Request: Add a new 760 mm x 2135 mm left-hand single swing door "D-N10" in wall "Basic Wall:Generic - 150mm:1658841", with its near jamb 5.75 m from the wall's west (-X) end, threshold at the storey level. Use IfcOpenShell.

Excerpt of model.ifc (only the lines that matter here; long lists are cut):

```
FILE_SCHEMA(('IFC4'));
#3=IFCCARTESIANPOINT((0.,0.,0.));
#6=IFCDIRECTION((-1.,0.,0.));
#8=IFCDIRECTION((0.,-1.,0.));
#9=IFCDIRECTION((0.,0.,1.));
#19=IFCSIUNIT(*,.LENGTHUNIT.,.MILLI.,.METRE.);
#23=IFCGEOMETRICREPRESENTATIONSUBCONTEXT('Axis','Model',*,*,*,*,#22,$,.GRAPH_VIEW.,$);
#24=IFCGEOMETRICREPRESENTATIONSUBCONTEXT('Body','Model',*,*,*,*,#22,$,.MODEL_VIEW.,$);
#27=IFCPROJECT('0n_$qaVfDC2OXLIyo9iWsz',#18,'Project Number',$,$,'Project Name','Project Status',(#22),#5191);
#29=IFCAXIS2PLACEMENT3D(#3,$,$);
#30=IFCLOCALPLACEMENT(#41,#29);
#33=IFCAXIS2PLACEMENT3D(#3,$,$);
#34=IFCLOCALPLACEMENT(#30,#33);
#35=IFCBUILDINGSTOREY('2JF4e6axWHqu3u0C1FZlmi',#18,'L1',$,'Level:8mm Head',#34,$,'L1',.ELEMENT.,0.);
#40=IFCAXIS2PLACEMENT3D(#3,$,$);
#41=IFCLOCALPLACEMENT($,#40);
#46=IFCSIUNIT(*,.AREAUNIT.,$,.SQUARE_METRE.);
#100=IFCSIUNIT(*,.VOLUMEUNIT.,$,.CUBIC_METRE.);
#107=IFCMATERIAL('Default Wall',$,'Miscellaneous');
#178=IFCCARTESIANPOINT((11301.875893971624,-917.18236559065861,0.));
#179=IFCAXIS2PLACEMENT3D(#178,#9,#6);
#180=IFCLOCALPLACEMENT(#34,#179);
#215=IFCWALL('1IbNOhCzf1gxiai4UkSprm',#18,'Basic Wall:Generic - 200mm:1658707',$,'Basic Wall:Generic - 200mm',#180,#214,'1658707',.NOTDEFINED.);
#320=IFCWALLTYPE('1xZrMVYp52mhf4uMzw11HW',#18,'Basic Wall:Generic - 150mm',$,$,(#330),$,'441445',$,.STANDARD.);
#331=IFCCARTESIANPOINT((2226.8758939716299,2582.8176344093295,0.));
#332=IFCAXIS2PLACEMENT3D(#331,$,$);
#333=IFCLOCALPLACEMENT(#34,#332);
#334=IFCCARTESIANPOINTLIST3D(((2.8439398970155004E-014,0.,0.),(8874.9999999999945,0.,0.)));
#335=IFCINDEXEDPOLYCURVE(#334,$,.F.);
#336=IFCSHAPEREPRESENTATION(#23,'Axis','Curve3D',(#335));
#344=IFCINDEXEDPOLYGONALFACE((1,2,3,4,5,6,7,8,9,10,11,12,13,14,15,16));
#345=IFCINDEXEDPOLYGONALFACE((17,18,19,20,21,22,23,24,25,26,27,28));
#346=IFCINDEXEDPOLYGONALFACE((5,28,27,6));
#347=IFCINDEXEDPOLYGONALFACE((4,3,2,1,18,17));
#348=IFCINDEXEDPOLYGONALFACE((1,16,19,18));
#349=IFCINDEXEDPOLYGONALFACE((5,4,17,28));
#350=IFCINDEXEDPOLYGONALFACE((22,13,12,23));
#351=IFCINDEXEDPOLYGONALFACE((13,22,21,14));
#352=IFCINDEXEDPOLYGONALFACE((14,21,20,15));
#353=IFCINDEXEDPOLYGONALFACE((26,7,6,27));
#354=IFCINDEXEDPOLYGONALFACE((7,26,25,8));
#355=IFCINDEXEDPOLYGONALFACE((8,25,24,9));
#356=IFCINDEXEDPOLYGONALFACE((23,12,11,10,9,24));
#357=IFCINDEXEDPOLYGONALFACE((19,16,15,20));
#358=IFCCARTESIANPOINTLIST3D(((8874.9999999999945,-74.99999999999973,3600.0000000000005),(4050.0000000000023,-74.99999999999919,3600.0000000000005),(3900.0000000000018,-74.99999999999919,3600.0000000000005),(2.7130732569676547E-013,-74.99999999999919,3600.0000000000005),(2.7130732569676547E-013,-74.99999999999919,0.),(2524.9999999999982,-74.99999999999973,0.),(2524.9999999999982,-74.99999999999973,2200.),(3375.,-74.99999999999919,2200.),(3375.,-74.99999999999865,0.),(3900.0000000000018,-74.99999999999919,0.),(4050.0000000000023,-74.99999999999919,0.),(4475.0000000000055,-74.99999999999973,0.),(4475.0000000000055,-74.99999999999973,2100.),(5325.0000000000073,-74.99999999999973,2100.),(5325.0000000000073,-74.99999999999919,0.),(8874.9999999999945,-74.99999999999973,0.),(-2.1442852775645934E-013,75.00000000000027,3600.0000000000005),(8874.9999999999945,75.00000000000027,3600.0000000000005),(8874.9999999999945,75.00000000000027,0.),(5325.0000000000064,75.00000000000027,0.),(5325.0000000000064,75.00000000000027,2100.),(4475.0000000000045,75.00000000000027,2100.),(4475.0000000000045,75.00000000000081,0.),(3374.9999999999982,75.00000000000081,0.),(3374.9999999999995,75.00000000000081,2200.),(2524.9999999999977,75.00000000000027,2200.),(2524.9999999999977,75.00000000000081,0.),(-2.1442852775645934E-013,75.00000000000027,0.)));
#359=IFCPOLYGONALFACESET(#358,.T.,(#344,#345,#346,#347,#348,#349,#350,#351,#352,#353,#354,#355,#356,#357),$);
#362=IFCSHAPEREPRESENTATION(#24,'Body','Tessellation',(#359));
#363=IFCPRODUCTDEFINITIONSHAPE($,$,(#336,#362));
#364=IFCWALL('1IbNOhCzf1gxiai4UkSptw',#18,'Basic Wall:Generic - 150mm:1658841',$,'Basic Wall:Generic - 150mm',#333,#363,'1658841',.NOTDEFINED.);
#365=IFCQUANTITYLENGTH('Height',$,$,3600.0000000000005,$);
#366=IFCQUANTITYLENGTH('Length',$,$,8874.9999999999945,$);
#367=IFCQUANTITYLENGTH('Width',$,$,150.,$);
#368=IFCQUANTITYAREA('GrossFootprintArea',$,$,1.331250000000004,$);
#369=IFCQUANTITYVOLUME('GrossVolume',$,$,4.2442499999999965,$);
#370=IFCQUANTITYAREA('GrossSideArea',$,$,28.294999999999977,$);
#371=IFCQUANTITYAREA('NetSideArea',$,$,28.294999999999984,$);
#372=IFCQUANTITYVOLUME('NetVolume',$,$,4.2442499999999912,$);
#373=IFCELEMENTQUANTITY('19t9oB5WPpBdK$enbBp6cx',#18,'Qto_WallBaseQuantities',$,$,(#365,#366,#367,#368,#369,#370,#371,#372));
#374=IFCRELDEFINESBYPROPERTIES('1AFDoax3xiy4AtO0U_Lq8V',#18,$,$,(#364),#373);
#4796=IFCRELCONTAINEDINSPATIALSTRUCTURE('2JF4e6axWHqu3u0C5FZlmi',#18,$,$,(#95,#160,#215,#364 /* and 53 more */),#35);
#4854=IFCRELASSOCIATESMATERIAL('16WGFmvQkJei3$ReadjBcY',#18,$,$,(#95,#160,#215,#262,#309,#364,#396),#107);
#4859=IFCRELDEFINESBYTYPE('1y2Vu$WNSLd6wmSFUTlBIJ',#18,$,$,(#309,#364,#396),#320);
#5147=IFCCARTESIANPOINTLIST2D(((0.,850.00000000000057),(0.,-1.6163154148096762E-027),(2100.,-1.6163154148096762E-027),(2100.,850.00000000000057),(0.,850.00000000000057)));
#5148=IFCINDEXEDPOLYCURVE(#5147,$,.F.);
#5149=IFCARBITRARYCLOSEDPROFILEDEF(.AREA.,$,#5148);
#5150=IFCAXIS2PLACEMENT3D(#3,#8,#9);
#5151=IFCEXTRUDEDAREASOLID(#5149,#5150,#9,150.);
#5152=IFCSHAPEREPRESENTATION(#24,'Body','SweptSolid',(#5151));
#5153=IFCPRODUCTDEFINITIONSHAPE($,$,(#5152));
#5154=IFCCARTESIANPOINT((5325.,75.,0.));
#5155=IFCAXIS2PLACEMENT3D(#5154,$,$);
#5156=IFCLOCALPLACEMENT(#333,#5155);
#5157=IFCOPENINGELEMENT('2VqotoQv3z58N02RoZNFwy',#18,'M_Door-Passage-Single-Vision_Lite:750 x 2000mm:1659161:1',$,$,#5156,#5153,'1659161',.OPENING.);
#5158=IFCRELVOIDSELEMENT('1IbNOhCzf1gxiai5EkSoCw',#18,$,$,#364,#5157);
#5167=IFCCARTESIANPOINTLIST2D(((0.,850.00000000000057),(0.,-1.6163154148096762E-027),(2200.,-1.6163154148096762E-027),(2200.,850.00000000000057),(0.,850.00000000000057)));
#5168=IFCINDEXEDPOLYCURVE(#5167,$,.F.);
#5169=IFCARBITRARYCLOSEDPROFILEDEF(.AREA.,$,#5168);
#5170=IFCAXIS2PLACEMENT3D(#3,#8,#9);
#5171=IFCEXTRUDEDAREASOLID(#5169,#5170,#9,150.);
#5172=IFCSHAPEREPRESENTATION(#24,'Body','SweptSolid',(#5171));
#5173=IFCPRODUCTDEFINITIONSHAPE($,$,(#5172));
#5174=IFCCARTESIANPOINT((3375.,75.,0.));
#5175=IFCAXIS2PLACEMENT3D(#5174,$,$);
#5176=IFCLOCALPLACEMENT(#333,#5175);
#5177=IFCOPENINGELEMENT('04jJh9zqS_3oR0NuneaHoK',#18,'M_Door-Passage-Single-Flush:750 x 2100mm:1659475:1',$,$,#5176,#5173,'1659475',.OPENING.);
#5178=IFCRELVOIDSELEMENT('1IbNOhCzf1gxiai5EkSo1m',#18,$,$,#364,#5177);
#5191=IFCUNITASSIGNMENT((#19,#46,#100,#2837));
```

```python
import numpy as np
import ifcopenshell
import ifcopenshell.api.feature
import ifcopenshell.api.geometry
import ifcopenshell.api.pset
import ifcopenshell.api.root
import ifcopenshell.api.spatial
import ifcopenshell.geom
import ifcopenshell.util.element
import ifcopenshell.util.placement
import ifcopenshell.util.representation
import ifcopenshell.util.shape
import ifcopenshell.util.unit

model = ifcopenshell.open("model.ifc")
unit_scale = ifcopenshell.util.unit.calculate_unit_scale(model)
area_scale = ifcopenshell.util.unit.calculate_unit_scale(model, "AREAUNIT")
volume_scale = ifcopenshell.util.unit.calculate_unit_scale(model, "VOLUMEUNIT")
settings = ifcopenshell.geom.settings()


def volume(element):
    """Net volume in cubic metres, openings subtracted."""
    shape = ifcopenshell.geom.create_shape(settings, element)
    return ifcopenshell.util.shape.get_volume(shape.geometry)


wall = model.by_guid("1IbNOhCzf1gxiai4UkSptw")
storey = ifcopenshell.util.element.get_container(wall, ifc_class="IfcBuildingStorey")
context = ifcopenshell.util.representation.get_context(model, "Model", "Body", "MODEL_VIEW")
before = volume(wall)

width, height, from_end, sill = 0.76, 2.135, 5.75, 0.0  # metres

# The wall runs along its own X axis, and the end named is its -X end.
wall_shape = ifcopenshell.geom.create_shape(settings, wall)
x, y, z = ifcopenshell.util.shape.get_vertices(wall_shape.geometry).T
start = x.min() + from_end
face, thickness = float(y.min()), float(y.max() - y.min())
wall_matrix = ifcopenshell.util.placement.get_local_placement(wall.ObjectPlacement)
level = ifcopenshell.util.placement.get_local_placement(storey.ObjectPlacement)[2, 3]


def in_wall(x, y):
    """Placement at x, y metres in the wall's axes, at sill height."""
    matrix = wall_matrix.copy()
    matrix[:, 3] = wall_matrix @ np.array([x / unit_scale, y / unit_scale, 0.0, 1.0])
    matrix[2, 3] = level + sill / unit_scale
    return matrix


# Opening: a box that overshoots both wall faces by 50 mm.
opening = ifcopenshell.api.root.create_entity(model, ifc_class="IfcOpeningElement", predefined_type="OPENING")
box = ifcopenshell.api.geometry.add_wall_representation(
    model, context=context, length=width, height=height, thickness=thickness + 0.1
)
ifcopenshell.api.geometry.assign_representation(model, product=opening, representation=box)
ifcopenshell.api.geometry.edit_object_placement(model, product=opening, matrix=in_wall(start, face - 0.05), is_si=False)
ifcopenshell.api.feature.add_feature(model, feature=opening, element=wall)

door = ifcopenshell.api.root.create_entity(model, ifc_class="IfcDoor", name="D-N10", predefined_type="DOOR")
door.OverallWidth, door.OverallHeight = width / unit_scale, height / unit_scale
door.OperationType = "SINGLE_SWING_LEFT"
body = ifcopenshell.api.geometry.add_door_representation(
    model,
    context=context,
    overall_width=door.OverallWidth,
    overall_height=door.OverallHeight,
    operation_type="SINGLE_SWING_LEFT",
    lining_properties={"LiningDepth": thickness / unit_scale, "ThresholdDepth": thickness / unit_scale},
)
ifcopenshell.api.geometry.assign_representation(model, product=door, representation=body)
ifcopenshell.api.spatial.assign_container(model, products=[door], relating_structure=storey)
ifcopenshell.api.feature.add_filling(model, opening=opening, element=door)

# The lining spans the wall, so the door starts at the wall face.
ifcopenshell.api.geometry.edit_object_placement(model, product=door, matrix=in_wall(start, face), is_si=False)

after = volume(wall)

# Update the wall's stored quantities.
qto = model.by_id(ifcopenshell.util.element.get_pset(wall, "Qto_WallBaseQuantities", should_inherit=False)["id"])
ifcopenshell.api.pset.edit_qto(model, qto=qto, properties={
    "NetSideArea": after / thickness / area_scale,
    "NetVolume": after / volume_scale,
})

print(f"wall volume {before:.3f} -> {after:.3f} m3")

model.write("model_edited.ifc")
```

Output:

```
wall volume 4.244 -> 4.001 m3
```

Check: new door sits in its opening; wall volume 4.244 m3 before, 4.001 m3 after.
